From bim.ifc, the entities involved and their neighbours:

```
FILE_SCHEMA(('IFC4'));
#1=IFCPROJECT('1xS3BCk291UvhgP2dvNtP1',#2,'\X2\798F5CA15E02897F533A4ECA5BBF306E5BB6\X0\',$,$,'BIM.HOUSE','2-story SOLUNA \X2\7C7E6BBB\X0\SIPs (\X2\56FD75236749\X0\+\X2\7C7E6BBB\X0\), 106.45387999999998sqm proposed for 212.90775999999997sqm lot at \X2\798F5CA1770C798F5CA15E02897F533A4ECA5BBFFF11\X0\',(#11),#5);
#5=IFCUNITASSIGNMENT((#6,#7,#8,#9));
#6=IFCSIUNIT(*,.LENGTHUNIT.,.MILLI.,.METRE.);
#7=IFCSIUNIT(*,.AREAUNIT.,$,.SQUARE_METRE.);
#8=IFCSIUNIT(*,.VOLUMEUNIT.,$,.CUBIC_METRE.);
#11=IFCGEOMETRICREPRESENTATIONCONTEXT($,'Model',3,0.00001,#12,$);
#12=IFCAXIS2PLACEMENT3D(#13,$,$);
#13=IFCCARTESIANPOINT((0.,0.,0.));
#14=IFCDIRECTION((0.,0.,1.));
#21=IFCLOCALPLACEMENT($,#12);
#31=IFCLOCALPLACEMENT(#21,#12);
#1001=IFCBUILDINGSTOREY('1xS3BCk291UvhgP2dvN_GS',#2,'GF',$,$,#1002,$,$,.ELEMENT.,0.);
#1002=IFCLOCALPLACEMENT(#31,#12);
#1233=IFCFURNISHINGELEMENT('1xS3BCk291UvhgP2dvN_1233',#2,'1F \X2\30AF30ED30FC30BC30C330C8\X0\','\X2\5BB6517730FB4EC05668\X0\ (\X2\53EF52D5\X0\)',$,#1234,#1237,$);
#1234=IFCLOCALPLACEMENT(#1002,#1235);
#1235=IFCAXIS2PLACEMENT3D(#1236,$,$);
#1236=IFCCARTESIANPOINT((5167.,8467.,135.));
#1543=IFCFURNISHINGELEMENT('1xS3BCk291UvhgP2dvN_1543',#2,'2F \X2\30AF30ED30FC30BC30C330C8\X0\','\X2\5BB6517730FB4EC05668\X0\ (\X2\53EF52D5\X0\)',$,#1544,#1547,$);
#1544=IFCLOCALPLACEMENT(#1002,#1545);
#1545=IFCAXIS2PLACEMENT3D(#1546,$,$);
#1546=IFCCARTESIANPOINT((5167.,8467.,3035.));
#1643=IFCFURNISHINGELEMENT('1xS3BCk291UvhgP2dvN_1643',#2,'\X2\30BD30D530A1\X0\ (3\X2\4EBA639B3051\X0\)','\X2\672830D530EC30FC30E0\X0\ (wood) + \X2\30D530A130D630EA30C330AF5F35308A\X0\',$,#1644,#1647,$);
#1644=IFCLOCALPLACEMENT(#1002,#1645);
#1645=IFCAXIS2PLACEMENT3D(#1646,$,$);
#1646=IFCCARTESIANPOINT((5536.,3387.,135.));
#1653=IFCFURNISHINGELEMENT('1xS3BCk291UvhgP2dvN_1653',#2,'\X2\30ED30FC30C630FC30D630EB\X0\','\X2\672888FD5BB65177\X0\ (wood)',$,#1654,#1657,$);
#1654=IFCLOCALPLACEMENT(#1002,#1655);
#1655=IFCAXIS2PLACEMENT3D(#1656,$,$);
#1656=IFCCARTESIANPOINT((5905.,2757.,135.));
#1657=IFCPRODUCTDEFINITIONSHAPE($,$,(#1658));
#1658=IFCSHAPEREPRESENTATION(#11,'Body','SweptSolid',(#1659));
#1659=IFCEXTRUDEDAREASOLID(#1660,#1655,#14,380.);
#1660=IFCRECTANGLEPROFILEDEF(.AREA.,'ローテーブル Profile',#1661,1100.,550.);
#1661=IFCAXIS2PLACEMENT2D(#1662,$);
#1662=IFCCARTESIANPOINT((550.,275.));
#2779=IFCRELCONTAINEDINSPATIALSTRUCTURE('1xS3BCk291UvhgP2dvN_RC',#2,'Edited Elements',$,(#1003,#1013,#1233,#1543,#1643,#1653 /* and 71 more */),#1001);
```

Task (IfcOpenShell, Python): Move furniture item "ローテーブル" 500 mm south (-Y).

```python
import ifcopenshell
import ifcopenshell.api.geometry
import ifcopenshell.util.placement

model = ifcopenshell.open("bim.ifc")

item = model.by_guid("1xS3BCk291UvhgP2dvN_1653")
matrix = ifcopenshell.util.placement.get_local_placement(item.ObjectPlacement)
matrix[1, 3] -= 500.0
ifcopenshell.api.geometry.edit_object_placement(model, product=item, matrix=matrix, is_si=False)

print(ifcopenshell.util.placement.get_local_placement(item.ObjectPlacement).round(3) + 0.0)

model.write("bim_updated.ifc")
```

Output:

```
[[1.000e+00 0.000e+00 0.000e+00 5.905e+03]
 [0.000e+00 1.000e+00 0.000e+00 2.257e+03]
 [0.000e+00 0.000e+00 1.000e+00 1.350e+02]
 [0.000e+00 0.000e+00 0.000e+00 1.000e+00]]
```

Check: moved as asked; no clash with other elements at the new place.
